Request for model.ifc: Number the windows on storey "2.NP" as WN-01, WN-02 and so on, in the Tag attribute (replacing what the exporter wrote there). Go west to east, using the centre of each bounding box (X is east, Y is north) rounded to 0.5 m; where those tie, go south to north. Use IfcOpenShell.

First a look at what the model holds.

```python
import ifcopenshell
import ifcopenshell.util.element
import ifcopenshell.util.placement

model = ifcopenshell.open("model.ifc")
print(model.schema)
storey = next(s for s in model.by_type("IfcBuildingStorey") if s.Name == "2.NP")
windows = [e for e in ifcopenshell.util.element.get_decomposition(storey) if e.is_a("IfcWindow")]
for e in sorted(windows, key=lambda e: e.id()):
    origin = ifcopenshell.util.placement.get_local_placement(e.ObjectPlacement)[:3, 3]
    print(e.id(), e.Tag, e.Name, origin.round(2) + 0.0, sep=" | ")
```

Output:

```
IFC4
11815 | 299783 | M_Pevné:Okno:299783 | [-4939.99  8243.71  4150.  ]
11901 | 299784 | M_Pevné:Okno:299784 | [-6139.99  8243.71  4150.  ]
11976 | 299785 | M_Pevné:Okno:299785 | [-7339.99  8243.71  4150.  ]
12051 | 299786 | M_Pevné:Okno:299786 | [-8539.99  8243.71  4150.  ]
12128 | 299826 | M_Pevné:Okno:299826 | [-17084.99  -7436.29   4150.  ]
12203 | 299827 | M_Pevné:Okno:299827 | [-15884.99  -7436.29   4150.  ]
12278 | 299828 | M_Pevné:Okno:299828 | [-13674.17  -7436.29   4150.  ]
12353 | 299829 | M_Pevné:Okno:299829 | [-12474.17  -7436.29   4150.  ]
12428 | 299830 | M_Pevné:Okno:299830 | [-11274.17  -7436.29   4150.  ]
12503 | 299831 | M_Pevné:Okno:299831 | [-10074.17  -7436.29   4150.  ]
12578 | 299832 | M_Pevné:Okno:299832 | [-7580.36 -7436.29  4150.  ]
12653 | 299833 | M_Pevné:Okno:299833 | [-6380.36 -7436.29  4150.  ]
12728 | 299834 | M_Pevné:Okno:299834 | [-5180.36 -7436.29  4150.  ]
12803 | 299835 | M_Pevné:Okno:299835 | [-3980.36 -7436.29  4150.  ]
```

```python
import ifcopenshell
import ifcopenshell.geom
import ifcopenshell.util.element
import ifcopenshell.util.shape

model = ifcopenshell.open("model.ifc")
settings = ifcopenshell.geom.settings()
settings.set("use-world-coords", True)


def centre(element):
    shape = ifcopenshell.geom.create_shape(settings, element)
    return ifcopenshell.util.shape.get_bbox_centroid(shape.geometry)


storey = next(s for s in model.by_type("IfcBuildingStorey") if s.Name == "2.NP")
windows = [e for e in ifcopenshell.util.element.get_decomposition(storey) if e.is_a("IfcWindow")]

# Insertion points can sit at a corner or the storey origin, so sort by the geometry (in metres).
centres = {e: centre(e) for e in windows}
windows.sort(key=lambda e: (round(centres[e][0] / 0.5), centres[e][1]))

for i, e in enumerate(windows, start=1):
    number = f"WN-{i:02d}"
    e.Tag = number
    print(e.id(), number)

model.write("model-out.ifc")
```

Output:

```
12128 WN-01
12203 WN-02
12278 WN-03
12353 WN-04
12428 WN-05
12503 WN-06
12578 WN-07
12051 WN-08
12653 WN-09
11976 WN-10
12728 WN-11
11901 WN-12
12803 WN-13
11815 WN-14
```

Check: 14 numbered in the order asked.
